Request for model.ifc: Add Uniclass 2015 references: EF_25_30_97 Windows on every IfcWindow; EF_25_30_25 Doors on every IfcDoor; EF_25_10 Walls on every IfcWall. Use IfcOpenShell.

First a look at what the model holds.

```python
import ifcopenshell

model = ifcopenshell.open("model.ifc")
print(model.schema)
print("classifications:", [c.Name for c in model.by_type("IfcClassification")])
for ifc_class in ("IfcDoor", "IfcRoof", "IfcStair", "IfcWall", "IfcWindow"):
    print(ifc_class, len(model.by_type(ifc_class)))
```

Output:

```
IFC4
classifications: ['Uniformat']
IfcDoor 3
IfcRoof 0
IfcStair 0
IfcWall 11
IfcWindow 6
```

```python
import ifcopenshell
import ifcopenshell.api.classification

model = ifcopenshell.open("model.ifc")

system = ifcopenshell.api.classification.add_classification(model, classification="Uniclass 2015")

codes = {
    "IfcWindow": ("EF_25_30_97", "Windows"),
    "IfcDoor": ("EF_25_30_25", "Doors"),
    "IfcWall": ("EF_25_10", "Walls"),
}
for ifc_class, (code, name) in codes.items():
    products = model.by_type(ifc_class)
    ifcopenshell.api.classification.add_reference(
        model, products=products, classification=system, identification=code, name=name
    )
    print(code, len(products))

model.write("model_edited.ifc")
```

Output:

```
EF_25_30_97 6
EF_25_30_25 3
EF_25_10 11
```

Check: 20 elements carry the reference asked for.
